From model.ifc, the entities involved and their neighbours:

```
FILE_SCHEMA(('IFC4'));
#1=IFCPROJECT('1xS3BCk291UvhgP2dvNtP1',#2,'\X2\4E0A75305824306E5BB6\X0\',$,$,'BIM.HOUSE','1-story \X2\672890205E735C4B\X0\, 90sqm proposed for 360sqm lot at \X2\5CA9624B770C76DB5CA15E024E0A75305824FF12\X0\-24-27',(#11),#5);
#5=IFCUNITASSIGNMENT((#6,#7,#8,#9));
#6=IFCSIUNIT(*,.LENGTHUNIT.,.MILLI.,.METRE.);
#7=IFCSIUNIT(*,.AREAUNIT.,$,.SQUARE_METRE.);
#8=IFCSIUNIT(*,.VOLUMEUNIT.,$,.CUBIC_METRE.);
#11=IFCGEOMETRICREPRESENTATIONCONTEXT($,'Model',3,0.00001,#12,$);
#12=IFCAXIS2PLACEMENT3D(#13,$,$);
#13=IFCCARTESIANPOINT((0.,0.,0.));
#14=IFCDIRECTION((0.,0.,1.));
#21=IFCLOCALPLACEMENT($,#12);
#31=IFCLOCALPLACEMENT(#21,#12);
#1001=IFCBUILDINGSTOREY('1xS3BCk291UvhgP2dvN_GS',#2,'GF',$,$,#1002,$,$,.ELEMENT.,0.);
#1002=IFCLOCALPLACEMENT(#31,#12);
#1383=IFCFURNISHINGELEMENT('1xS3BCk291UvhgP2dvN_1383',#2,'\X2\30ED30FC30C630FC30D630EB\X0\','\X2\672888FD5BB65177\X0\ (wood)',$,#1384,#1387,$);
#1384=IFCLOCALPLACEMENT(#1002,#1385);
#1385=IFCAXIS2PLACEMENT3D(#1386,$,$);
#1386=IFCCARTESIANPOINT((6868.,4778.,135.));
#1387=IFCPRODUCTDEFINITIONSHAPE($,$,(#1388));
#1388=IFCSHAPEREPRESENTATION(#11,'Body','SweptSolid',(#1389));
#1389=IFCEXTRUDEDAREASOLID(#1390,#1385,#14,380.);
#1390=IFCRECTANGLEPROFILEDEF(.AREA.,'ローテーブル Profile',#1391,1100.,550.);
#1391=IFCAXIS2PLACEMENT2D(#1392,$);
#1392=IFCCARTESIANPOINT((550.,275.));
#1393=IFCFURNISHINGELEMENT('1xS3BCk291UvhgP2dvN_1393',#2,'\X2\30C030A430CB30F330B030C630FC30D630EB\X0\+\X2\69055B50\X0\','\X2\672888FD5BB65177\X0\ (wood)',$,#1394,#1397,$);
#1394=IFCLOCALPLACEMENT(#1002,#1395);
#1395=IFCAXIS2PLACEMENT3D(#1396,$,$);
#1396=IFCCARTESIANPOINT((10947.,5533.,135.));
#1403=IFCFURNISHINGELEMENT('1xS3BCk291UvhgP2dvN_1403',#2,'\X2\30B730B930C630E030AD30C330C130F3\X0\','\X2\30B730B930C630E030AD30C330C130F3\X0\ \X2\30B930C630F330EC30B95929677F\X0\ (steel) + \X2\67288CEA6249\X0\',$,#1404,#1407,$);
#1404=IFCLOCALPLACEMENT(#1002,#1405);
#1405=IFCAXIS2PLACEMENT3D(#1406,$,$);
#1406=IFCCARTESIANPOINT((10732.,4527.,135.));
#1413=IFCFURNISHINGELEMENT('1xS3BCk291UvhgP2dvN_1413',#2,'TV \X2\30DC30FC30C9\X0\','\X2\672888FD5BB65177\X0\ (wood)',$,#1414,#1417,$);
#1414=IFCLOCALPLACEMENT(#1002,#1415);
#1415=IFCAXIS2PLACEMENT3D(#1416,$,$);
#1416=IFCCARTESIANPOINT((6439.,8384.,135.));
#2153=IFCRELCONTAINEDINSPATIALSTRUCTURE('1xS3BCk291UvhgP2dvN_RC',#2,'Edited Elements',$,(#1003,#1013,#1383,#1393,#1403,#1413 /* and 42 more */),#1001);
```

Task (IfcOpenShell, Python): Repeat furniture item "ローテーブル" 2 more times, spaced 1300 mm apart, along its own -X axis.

```python
import ifcopenshell
import ifcopenshell.api.geometry
import ifcopenshell.api.root
import ifcopenshell.util.element
import ifcopenshell.util.placement

model = ifcopenshell.open("model.ifc")


def reuse_history(source, copy):
    """copy_class also copies each property set's owner history, people and application; keep the originals."""
    for rel in copy.IsDefinedBy:
        if rel.is_a("IfcRelDefinesByProperties") and (history := rel.RelatingPropertyDefinition.OwnerHistory):
            rel.RelatingPropertyDefinition.OwnerHistory = source.OwnerHistory
            ifcopenshell.util.element.remove_deep2(model, history)


source = model.by_guid("1xS3BCk291UvhgP2dvN_1383")
base = ifcopenshell.util.placement.get_local_placement(source.ObjectPlacement)
step = -base[:3, 0] * 1300.0

for i in range(1, 3):
    copy = ifcopenshell.api.root.copy_class(model, product=source)
    copy.Representation = ifcopenshell.util.element.copy_deep(
        model, source.Representation, exclude=["IfcGeometricRepresentationContext", "IfcRepresentationMap"]
    )
    reuse_history(source, copy)
    matrix = base.copy()
    matrix[:3, 3] += i * step
    print("added at", matrix[:3, 3].round(3) + 0.0)
    ifcopenshell.api.geometry.edit_object_placement(model, product=copy, matrix=matrix, is_si=False)

model.write("model_updated.ifc")
```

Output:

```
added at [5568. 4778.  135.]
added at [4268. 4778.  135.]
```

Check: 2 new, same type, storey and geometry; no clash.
